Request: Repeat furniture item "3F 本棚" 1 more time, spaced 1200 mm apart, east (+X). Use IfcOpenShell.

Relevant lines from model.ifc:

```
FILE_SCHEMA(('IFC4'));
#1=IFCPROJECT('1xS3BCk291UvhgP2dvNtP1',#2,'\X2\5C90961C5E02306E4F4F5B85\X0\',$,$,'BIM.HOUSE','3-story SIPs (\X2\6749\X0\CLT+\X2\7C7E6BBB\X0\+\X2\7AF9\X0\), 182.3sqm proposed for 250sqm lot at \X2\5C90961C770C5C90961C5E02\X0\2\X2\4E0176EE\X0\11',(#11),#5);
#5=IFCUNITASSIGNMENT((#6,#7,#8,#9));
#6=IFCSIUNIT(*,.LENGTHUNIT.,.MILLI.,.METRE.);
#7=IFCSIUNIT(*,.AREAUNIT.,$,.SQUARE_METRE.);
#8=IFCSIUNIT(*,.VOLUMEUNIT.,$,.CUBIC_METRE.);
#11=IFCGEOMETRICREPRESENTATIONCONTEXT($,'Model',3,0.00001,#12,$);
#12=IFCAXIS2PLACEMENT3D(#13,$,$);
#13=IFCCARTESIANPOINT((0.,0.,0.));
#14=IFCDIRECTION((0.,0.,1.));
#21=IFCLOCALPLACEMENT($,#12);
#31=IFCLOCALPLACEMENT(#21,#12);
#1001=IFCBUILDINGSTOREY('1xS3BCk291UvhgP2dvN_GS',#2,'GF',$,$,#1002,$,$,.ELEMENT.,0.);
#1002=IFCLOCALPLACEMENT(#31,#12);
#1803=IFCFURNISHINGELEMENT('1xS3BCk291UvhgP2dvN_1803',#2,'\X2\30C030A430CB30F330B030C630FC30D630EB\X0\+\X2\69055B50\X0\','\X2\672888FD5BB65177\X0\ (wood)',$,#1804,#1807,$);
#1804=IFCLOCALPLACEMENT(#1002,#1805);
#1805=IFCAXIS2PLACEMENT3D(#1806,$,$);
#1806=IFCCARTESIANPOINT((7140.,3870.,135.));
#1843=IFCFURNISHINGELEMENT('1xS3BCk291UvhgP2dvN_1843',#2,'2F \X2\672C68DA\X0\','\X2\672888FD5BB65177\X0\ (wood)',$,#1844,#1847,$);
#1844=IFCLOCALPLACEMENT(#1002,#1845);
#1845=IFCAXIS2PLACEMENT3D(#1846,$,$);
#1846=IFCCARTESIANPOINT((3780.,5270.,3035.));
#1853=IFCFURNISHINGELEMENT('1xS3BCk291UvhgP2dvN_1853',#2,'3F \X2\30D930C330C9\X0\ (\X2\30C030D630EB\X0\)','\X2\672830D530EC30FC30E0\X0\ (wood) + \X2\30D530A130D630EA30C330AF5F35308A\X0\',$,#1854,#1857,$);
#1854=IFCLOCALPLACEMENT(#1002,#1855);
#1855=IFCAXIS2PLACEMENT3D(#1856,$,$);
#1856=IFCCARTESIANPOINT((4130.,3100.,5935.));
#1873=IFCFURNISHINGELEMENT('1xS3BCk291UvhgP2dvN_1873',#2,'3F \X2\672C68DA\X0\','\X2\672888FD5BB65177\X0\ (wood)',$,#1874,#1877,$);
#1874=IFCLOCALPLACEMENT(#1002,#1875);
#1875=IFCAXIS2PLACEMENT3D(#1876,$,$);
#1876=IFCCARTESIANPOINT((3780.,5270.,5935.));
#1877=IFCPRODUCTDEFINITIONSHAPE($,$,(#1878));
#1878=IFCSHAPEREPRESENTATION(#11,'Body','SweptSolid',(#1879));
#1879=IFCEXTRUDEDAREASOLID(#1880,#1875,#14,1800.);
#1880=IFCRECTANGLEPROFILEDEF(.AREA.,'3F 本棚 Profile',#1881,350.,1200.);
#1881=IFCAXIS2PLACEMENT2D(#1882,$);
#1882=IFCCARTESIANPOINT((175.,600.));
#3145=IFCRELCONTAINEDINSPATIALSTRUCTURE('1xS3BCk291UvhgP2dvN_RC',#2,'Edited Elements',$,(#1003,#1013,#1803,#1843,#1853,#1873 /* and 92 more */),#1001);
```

```python
import numpy as np
import ifcopenshell
import ifcopenshell.api.geometry
import ifcopenshell.api.root
import ifcopenshell.util.element
import ifcopenshell.util.placement
import ifcopenshell.util.unit

model = ifcopenshell.open("model.ifc")
unit_scale = ifcopenshell.util.unit.calculate_unit_scale(model)


def reuse_history(source, copy):
    """copy_class also copies each property set's owner history, people and application; keep the originals."""
    for rel in copy.IsDefinedBy:
        if rel.is_a("IfcRelDefinesByProperties") and (history := rel.RelatingPropertyDefinition.OwnerHistory):
            rel.RelatingPropertyDefinition.OwnerHistory = source.OwnerHistory
            ifcopenshell.util.element.remove_deep2(model, history)


source = model.by_id(1873)
base = ifcopenshell.util.placement.get_local_placement(source.ObjectPlacement)
step = np.array([1.0, 0.0, 0.0]) * 1.2 / unit_scale

for i in range(1, 2):
    copy = ifcopenshell.api.root.copy_class(model, product=source)
    copy.Representation = ifcopenshell.util.element.copy_deep(
        model, source.Representation, exclude=["IfcGeometricRepresentationContext", "IfcRepresentationMap"]
    )
    reuse_history(source, copy)
    matrix = base.copy()
    matrix[:3, 3] += i * step
    print("added at", matrix[:3, 3].round(3) + 0.0)
    ifcopenshell.api.geometry.edit_object_placement(model, product=copy, matrix=matrix, is_si=False)

model.write("model_updated.ifc")
```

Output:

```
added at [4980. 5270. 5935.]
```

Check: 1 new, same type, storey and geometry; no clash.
